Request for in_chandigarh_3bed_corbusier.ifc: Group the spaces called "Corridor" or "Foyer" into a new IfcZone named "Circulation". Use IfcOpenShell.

First a look at what the model holds.

```python
import ifcopenshell

model = ifcopenshell.open("in_chandigarh_3bed_corbusier.ifc")
print(model.schema)
seen = {}
for space in model.by_type("IfcSpace"):
    seen[space.LongName] = seen.get(space.LongName, 0) + 1
for name, count in sorted(seen.items(), key=str):
    print(count, "x", name)
print("zones:", [z.Name for z in model.by_type("IfcZone")][:20])
```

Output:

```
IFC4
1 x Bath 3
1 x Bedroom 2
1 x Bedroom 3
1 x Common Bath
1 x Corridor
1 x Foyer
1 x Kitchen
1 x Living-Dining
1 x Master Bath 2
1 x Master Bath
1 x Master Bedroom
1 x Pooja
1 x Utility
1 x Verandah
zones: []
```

```python
import ifcopenshell
import ifcopenshell.api.group
import ifcopenshell.api.root

model = ifcopenshell.open("in_chandigarh_3bed_corbusier.ifc")

names = {"Corridor", "Foyer"}
spaces = [s for s in model.by_type("IfcSpace") if s.LongName in names]

zone = ifcopenshell.api.root.create_entity(model, ifc_class="IfcZone", name="Circulation")
ifcopenshell.api.group.assign_group(model, products=spaces, group=zone)
print(len(spaces), "spaces in", zone.Name)

model.write("in_chandigarh_3bed_corbusier-out.ifc")
```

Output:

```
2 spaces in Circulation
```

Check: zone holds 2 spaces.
